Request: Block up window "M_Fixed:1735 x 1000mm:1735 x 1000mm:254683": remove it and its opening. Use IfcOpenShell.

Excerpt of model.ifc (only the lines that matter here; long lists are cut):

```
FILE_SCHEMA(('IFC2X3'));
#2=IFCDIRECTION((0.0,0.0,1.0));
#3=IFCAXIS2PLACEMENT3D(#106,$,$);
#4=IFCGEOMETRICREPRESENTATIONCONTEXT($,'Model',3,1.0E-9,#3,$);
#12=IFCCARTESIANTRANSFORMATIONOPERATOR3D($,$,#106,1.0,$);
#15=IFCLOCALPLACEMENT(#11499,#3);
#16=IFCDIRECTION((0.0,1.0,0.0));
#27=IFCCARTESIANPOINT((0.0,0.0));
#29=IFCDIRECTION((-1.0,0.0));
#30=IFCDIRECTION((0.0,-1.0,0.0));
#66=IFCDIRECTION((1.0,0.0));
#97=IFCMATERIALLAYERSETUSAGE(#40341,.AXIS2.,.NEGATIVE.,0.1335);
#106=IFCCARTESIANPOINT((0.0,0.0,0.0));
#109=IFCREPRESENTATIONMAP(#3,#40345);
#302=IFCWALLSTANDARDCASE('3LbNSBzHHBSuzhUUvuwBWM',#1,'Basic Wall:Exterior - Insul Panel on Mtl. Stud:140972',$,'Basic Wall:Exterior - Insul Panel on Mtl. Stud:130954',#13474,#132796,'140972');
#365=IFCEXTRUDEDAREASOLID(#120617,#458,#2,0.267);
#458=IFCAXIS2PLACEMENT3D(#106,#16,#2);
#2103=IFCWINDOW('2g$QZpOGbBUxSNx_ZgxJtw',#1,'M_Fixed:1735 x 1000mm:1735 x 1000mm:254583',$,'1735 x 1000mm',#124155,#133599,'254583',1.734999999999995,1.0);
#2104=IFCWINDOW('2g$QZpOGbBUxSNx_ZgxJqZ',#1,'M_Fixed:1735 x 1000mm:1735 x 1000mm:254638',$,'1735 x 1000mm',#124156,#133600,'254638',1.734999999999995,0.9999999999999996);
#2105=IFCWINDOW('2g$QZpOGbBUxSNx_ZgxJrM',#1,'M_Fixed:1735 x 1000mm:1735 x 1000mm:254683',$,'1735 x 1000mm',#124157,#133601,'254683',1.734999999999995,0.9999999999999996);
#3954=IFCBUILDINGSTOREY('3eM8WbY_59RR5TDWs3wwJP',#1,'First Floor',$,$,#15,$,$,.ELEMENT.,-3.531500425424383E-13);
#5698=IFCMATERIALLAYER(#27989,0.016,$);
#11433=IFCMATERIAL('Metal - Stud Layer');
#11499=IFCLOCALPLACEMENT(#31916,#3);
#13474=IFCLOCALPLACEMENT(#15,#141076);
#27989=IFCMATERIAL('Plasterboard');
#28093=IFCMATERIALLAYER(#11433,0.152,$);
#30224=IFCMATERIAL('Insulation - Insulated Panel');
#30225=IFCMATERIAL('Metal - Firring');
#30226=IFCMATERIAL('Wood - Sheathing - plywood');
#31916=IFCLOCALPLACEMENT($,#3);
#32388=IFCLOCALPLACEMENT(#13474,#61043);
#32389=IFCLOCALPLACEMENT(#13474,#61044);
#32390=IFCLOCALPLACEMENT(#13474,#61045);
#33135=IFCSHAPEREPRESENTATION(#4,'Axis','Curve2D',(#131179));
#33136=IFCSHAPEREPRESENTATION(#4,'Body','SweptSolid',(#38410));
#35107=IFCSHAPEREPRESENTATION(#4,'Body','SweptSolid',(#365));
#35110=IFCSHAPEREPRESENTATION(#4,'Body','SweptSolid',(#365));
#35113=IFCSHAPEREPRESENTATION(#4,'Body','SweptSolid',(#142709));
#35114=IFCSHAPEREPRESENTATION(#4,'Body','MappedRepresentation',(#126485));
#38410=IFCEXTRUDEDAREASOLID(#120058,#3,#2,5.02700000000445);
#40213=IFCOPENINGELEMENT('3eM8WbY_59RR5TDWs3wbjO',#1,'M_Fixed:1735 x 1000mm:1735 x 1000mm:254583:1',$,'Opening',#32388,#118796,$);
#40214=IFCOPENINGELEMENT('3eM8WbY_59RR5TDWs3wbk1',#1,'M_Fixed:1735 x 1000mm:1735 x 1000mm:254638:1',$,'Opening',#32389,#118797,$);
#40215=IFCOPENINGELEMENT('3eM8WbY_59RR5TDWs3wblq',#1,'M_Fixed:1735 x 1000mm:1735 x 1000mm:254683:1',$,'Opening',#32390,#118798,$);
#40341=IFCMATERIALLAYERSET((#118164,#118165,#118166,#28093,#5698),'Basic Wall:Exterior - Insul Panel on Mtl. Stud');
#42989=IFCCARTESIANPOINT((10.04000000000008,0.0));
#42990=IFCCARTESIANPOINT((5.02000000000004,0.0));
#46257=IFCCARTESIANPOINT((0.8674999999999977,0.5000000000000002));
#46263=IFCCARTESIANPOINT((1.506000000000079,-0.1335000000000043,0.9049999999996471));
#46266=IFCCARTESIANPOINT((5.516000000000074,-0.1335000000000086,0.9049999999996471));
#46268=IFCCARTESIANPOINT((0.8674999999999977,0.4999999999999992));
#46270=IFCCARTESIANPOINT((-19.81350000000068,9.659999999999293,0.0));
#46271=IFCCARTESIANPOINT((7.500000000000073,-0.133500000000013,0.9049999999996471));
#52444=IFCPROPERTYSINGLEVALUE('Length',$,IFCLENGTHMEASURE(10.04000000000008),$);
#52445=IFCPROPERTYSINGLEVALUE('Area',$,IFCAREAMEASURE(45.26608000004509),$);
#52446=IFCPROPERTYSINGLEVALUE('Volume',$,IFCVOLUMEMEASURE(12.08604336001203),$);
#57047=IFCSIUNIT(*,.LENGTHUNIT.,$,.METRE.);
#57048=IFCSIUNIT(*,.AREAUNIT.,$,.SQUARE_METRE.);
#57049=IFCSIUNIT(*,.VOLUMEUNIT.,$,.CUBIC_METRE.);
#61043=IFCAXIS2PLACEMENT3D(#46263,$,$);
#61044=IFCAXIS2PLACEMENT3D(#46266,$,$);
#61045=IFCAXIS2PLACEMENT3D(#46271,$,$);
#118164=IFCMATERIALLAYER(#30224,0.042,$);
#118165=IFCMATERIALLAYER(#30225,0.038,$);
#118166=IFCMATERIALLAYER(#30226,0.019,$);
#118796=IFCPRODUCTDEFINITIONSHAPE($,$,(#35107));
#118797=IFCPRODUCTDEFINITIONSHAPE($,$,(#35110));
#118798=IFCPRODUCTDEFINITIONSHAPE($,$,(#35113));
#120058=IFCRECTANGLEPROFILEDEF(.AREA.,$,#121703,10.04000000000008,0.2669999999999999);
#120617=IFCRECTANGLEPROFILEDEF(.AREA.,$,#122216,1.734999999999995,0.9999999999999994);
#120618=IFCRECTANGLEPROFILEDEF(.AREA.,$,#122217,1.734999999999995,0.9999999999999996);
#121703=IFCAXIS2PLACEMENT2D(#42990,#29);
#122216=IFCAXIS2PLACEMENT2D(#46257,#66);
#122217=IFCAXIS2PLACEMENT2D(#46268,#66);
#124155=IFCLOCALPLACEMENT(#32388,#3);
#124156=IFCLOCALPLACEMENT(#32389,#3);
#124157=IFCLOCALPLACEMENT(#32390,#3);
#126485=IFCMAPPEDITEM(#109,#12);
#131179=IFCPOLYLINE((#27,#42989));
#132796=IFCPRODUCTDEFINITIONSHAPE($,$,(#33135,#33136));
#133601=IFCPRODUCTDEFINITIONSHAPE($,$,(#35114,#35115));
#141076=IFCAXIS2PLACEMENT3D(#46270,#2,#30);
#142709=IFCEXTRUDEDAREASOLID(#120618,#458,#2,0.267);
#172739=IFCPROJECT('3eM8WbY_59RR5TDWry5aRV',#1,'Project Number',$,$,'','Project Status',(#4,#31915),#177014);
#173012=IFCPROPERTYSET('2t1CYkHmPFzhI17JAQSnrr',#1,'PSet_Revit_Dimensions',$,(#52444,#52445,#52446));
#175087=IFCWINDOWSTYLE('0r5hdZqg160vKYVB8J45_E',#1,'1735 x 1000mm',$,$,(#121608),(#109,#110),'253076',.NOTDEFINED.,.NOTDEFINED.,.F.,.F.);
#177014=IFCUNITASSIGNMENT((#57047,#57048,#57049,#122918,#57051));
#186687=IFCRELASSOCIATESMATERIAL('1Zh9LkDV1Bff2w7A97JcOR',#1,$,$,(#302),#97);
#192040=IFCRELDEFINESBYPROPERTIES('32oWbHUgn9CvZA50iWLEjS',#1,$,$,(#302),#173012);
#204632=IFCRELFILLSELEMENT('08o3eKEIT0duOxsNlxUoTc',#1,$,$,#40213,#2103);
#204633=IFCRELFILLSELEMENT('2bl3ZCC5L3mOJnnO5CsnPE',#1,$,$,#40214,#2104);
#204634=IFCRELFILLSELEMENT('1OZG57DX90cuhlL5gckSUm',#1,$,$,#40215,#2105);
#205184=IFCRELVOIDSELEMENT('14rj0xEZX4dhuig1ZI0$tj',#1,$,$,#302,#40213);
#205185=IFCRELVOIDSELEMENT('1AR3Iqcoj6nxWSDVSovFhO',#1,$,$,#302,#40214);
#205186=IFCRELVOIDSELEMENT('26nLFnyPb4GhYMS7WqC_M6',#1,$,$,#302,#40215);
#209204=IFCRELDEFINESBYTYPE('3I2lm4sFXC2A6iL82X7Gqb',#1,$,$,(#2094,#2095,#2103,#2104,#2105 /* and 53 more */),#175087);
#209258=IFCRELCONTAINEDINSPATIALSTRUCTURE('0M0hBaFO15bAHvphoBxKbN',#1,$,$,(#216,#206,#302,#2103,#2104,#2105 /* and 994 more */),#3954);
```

```python
import ifcopenshell
import ifcopenshell.api.feature
import ifcopenshell.api.pset
import ifcopenshell.api.root
import ifcopenshell.geom
import ifcopenshell.util.element
import ifcopenshell.util.shape
import ifcopenshell.util.unit

model = ifcopenshell.open("model.ifc")
area_scale = ifcopenshell.util.unit.calculate_unit_scale(model, "AREAUNIT")
volume_scale = ifcopenshell.util.unit.calculate_unit_scale(model, "VOLUMEUNIT")
settings = ifcopenshell.geom.settings()


def volume(element):
    """Net volume in cubic metres, openings subtracted."""
    shape = ifcopenshell.geom.create_shape(settings, element)
    return ifcopenshell.util.shape.get_volume(shape.geometry)


window = model.by_guid("2g$QZpOGbBUxSNx_ZgxJrM")
opening = window.FillsVoids[0].RelatingOpeningElement
wall = opening.VoidsElements[0].RelatingBuildingElement
before = volume(wall)

ifcopenshell.api.root.remove_product(model, product=window)
ifcopenshell.api.feature.remove_feature(model, feature=opening)

after = volume(wall)
thickness = 0.267  # wall thickness in metres

# Update the wall's stored quantities.
pset = model.by_id(ifcopenshell.util.element.get_pset(wall, "PSet_Revit_Dimensions", should_inherit=False)["id"])
ifcopenshell.api.pset.edit_pset(model, pset=pset, properties={
    "Area": model.create_entity("IfcAreaMeasure", after / thickness / area_scale),
    "Volume": model.create_entity("IfcVolumeMeasure", after / volume_scale),
})

print(f"wall volume {before:.3f} -> {after:.3f} m3")

model.write("model_rev.ifc")
```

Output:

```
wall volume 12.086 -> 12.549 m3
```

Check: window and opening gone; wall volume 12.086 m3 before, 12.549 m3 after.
